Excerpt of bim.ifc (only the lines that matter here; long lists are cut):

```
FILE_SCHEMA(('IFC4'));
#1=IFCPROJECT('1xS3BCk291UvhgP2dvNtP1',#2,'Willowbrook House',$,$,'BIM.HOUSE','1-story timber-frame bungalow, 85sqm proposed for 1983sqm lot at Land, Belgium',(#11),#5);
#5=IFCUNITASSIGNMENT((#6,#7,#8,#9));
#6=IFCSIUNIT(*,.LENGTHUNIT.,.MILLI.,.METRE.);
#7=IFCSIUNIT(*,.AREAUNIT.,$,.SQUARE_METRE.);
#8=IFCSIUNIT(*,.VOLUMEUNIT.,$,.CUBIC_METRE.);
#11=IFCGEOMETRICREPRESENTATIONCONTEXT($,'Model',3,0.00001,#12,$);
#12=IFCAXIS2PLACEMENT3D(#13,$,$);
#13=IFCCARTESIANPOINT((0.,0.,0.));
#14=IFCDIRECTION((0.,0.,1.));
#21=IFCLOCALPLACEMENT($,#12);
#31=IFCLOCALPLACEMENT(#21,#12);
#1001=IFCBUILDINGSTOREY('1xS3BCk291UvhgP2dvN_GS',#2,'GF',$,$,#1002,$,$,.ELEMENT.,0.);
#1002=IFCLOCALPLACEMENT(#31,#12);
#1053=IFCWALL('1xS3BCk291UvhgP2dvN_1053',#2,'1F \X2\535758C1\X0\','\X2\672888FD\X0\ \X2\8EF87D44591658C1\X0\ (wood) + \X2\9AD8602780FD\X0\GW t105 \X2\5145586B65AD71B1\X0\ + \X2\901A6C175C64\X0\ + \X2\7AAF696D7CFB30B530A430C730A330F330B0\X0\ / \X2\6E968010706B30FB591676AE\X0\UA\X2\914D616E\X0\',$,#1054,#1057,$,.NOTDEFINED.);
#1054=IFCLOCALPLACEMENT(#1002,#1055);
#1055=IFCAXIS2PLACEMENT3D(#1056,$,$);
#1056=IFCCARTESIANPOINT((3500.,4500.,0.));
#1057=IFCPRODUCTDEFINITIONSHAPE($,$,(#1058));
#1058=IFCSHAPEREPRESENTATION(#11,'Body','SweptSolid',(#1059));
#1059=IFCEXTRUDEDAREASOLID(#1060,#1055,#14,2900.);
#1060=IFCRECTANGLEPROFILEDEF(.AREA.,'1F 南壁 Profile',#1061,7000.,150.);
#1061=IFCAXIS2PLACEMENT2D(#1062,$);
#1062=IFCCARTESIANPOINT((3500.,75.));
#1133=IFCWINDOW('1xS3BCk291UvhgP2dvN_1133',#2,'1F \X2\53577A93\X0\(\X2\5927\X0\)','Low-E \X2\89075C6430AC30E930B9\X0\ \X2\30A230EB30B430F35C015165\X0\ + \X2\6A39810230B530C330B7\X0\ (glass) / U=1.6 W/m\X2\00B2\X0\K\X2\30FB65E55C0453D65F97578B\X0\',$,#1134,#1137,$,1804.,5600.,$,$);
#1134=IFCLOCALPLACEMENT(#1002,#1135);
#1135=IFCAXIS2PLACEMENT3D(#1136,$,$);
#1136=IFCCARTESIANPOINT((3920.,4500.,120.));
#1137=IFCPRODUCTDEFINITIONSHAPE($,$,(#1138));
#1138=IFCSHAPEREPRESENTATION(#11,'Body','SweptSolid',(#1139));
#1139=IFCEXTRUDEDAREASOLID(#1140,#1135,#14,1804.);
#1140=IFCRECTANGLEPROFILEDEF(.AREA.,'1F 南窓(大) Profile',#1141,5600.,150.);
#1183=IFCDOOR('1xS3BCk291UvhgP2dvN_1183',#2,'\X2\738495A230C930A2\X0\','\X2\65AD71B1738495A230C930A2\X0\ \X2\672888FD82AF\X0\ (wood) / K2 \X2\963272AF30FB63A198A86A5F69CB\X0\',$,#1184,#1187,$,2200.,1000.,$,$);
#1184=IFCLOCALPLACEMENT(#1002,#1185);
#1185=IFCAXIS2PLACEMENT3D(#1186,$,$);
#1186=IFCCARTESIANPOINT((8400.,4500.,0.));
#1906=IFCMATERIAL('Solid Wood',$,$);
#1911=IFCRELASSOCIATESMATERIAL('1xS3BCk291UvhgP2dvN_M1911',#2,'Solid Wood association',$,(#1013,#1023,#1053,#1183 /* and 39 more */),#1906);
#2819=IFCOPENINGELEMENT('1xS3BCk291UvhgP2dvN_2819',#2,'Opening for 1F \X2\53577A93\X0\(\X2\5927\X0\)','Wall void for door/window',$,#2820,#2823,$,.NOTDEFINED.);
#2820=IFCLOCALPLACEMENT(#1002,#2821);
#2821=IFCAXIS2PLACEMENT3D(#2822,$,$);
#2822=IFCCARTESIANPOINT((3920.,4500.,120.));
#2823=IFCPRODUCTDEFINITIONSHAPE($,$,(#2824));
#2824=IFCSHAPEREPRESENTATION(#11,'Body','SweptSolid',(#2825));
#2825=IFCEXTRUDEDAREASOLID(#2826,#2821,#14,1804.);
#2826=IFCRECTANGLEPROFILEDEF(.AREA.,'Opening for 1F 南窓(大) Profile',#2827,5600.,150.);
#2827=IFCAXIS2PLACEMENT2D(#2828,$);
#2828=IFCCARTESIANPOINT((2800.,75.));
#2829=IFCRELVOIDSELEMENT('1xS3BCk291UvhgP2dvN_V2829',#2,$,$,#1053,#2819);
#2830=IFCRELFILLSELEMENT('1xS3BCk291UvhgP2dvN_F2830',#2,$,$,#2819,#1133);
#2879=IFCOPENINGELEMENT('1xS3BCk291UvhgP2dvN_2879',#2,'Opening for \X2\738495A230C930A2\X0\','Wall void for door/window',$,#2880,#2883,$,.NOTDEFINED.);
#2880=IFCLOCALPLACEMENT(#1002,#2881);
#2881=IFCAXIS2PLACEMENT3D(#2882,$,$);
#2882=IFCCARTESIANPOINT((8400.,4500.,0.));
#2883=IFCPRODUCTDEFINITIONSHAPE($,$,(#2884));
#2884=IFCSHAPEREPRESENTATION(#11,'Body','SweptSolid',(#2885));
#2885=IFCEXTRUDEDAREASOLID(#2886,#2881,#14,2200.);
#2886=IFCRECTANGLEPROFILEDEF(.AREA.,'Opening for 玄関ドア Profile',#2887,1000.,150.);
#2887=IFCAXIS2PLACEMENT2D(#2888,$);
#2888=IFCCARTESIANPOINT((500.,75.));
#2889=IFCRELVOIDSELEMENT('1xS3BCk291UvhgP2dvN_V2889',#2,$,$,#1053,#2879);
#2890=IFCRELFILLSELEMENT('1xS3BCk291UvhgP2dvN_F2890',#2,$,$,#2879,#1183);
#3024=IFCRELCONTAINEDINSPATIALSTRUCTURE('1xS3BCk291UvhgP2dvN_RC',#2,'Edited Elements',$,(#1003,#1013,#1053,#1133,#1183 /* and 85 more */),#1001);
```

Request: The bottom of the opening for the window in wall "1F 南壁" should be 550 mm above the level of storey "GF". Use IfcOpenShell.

```python
import numpy as np
import ifcopenshell
import ifcopenshell.api.geometry
import ifcopenshell.geom
import ifcopenshell.util.element
import ifcopenshell.util.placement
import ifcopenshell.util.shape
import ifcopenshell.util.unit

model = ifcopenshell.open("bim.ifc")
unit_scale = ifcopenshell.util.unit.calculate_unit_scale(model)

window = model.by_guid("1xS3BCk291UvhgP2dvN_1133")
opening = window.FillsVoids[0].RelatingOpeningElement
storey = ifcopenshell.util.element.get_container(window, ifc_class="IfcBuildingStorey")
level = ifcopenshell.util.placement.get_local_placement(storey.ObjectPlacement)[2, 3]

# The opening's origin need not be at the sill, so measure its lowest point.
shape = ifcopenshell.geom.create_shape(ifcopenshell.geom.settings(), opening)
bottom = ifcopenshell.util.shape.get_shape_bottom_elevation(shape, shape.geometry) / unit_scale
dz = level + 0.55 / unit_scale - bottom

shift = np.array([0.0, 0.0, dz])
# The window is not placed relative to its opening, so move both.
for product in (opening, window):
    matrix = ifcopenshell.util.placement.get_local_placement(product.ObjectPlacement)
    matrix[:3, 3] += shift
    ifcopenshell.api.geometry.edit_object_placement(model, product=product, matrix=matrix, is_si=False)

print(f"moved by {dz * unit_scale:+.3f} m")

model.write("bim_v2.ifc")
```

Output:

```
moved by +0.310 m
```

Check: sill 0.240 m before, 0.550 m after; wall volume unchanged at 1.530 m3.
